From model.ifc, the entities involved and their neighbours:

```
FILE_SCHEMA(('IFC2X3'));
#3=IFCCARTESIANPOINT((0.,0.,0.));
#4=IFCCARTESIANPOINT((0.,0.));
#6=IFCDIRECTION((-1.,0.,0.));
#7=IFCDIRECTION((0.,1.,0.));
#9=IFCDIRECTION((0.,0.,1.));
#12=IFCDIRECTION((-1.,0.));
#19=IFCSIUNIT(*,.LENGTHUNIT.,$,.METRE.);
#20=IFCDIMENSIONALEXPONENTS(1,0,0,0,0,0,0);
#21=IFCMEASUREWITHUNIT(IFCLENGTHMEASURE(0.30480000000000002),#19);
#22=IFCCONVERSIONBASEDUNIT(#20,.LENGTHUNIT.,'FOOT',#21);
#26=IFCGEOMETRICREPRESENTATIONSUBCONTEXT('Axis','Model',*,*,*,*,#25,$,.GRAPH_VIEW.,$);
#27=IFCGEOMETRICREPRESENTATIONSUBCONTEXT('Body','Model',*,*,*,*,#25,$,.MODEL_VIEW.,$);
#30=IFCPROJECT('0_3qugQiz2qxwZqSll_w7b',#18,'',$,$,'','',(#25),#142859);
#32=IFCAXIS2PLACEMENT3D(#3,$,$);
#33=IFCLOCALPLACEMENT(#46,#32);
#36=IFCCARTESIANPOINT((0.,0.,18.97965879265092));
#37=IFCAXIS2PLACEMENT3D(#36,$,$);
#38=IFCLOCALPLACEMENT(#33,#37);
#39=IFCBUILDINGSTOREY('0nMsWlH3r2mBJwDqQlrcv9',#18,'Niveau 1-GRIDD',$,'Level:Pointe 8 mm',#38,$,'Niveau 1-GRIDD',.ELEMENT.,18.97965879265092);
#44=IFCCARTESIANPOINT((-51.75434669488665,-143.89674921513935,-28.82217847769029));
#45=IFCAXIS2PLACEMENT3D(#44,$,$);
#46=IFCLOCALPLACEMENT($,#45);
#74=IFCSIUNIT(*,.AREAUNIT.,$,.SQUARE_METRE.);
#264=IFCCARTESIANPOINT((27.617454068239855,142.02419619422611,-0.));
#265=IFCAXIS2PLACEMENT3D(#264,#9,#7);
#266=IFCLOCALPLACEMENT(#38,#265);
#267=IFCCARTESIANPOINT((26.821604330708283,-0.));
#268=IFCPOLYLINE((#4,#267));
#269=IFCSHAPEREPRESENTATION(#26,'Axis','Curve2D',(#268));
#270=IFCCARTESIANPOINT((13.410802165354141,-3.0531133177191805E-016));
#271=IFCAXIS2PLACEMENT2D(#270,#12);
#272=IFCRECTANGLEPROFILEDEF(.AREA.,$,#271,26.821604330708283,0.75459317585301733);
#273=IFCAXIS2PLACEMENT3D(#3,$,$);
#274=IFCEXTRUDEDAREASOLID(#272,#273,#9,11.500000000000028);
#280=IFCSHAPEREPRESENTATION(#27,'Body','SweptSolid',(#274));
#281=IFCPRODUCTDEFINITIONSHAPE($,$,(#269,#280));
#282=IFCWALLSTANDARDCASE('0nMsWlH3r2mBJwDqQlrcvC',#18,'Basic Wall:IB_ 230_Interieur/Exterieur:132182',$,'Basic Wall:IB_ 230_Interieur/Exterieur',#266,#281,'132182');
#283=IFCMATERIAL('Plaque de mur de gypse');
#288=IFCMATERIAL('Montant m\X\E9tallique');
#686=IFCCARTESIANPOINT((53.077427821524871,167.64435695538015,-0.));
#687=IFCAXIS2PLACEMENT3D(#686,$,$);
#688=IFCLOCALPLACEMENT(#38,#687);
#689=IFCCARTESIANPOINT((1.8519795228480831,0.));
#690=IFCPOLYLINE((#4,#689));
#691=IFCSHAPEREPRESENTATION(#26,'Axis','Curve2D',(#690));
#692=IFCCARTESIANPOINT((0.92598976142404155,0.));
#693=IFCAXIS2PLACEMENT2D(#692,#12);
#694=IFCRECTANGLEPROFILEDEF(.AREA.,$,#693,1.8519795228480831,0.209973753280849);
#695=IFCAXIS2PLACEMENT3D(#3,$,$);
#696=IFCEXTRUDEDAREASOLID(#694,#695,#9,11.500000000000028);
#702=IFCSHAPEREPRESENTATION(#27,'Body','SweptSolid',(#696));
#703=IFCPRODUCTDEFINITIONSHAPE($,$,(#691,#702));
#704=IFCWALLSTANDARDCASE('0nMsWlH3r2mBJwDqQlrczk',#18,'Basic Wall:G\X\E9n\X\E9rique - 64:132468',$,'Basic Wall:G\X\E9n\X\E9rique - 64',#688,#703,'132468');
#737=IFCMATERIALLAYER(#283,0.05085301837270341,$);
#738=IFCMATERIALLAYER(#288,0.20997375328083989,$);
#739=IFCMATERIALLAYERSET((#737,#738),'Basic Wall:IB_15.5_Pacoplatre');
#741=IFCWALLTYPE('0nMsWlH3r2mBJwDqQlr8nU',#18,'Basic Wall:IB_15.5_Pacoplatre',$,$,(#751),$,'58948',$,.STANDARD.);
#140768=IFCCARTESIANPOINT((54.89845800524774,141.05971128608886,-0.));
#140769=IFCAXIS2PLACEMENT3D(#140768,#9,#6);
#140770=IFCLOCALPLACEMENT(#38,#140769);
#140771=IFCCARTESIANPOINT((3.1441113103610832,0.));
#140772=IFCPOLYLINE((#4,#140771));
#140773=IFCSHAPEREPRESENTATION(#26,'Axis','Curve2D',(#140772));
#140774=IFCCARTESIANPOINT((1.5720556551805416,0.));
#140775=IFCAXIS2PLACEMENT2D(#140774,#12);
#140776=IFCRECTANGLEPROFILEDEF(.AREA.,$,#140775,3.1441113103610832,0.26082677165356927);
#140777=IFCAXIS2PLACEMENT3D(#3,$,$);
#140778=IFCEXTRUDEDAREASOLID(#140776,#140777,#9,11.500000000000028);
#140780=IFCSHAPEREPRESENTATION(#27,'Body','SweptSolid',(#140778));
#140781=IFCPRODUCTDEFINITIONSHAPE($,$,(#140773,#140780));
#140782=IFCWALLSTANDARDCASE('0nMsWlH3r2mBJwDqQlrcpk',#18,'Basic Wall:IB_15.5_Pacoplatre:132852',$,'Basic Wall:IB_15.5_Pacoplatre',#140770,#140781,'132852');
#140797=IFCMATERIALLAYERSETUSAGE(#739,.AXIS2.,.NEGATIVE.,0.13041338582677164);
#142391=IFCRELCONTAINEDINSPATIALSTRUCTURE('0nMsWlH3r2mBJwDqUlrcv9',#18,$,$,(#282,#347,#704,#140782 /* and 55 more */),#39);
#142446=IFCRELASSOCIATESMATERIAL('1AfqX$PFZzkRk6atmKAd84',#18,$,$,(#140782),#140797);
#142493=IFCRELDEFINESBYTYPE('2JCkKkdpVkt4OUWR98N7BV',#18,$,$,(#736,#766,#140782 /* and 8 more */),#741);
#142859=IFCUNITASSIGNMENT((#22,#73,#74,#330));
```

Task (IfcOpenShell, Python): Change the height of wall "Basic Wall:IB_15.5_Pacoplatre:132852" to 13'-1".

```python
import ifcopenshell
import ifcopenshell.geom
import ifcopenshell.util.representation
import ifcopenshell.util.shape
import ifcopenshell.util.unit

model = ifcopenshell.open("model.ifc")
unit_scale = ifcopenshell.util.unit.calculate_unit_scale(model)
settings = ifcopenshell.geom.settings()


def volume(element):
    """Net volume in cubic metres, openings subtracted."""
    shape = ifcopenshell.geom.create_shape(settings, element)
    return ifcopenshell.util.shape.get_volume(shape.geometry)


wall = model.by_guid("0nMsWlH3r2mBJwDqQlrcpk")
before = volume(wall)

body = ifcopenshell.util.representation.get_representation(wall, "Model", "Body")
solid = body.Items[0]
old_height = solid.Depth
solid.Depth = 157 * 0.0254 / unit_scale
after = volume(wall)

print(f"height {old_height:g} -> {solid.Depth:g}, volume {before:.3f} -> {after:.3f} m3")

model.write("model_updated.ifc")
```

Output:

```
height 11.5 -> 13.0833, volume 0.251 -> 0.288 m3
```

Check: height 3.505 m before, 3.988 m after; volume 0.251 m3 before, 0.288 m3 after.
